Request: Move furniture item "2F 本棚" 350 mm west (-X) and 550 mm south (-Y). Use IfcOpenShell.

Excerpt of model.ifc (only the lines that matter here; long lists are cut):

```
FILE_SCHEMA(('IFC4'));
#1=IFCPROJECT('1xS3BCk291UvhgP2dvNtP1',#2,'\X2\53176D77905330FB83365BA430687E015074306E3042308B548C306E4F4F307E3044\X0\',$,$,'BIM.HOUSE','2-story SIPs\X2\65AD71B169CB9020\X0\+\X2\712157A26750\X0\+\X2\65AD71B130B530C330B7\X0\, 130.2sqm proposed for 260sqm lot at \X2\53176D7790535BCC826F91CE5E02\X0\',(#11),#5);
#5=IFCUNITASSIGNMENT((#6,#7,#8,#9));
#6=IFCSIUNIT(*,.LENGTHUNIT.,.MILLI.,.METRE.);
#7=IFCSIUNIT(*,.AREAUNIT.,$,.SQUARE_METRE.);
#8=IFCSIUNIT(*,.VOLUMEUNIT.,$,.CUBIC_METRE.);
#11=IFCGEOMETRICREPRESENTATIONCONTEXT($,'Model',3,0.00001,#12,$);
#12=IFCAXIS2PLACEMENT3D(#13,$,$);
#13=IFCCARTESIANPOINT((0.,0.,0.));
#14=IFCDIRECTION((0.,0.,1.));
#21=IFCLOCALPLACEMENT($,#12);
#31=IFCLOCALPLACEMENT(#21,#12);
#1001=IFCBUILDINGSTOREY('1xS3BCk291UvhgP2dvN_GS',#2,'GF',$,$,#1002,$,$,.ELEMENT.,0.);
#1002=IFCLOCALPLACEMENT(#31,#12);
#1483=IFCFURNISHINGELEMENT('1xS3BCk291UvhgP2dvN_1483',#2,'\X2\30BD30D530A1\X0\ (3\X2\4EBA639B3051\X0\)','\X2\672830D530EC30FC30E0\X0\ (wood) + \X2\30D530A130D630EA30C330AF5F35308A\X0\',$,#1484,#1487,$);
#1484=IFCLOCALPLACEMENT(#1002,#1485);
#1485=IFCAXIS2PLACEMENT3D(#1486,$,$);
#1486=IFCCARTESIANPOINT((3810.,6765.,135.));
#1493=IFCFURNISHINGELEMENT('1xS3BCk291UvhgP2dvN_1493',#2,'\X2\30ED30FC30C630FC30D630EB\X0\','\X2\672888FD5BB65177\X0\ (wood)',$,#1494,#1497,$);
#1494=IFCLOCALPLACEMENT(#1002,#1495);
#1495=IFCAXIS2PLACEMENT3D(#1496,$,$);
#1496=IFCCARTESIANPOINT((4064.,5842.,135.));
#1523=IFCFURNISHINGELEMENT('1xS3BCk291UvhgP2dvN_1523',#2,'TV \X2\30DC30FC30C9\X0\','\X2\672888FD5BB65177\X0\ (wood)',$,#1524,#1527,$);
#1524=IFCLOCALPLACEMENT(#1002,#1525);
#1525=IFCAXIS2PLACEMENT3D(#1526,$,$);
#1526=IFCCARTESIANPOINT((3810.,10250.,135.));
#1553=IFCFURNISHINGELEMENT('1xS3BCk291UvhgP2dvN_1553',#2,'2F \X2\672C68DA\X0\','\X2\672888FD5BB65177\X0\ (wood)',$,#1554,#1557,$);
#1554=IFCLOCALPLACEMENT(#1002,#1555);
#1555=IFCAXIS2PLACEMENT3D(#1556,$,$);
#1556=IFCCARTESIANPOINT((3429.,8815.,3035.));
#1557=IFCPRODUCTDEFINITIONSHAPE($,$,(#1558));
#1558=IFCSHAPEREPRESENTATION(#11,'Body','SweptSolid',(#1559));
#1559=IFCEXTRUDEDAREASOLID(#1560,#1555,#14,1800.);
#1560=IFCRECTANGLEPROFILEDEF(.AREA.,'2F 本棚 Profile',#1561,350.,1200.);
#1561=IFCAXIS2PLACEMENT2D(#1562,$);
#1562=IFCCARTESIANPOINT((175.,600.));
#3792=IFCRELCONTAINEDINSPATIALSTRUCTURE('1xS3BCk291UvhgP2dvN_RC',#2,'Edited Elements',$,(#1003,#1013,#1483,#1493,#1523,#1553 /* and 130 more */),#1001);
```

```python
import ifcopenshell
import ifcopenshell.api.geometry
import ifcopenshell.util.placement
import ifcopenshell.util.unit

model = ifcopenshell.open("model.ifc")
unit_scale = ifcopenshell.util.unit.calculate_unit_scale(model)

item = model.by_guid("1xS3BCk291UvhgP2dvN_1553")
matrix = ifcopenshell.util.placement.get_local_placement(item.ObjectPlacement)
matrix[0, 3] -= 0.35 / unit_scale
matrix[1, 3] -= 0.55 / unit_scale
ifcopenshell.api.geometry.edit_object_placement(model, product=item, matrix=matrix, is_si=False)

print(ifcopenshell.util.placement.get_local_placement(item.ObjectPlacement).round(3) + 0.0)

model.write("model-out.ifc")
```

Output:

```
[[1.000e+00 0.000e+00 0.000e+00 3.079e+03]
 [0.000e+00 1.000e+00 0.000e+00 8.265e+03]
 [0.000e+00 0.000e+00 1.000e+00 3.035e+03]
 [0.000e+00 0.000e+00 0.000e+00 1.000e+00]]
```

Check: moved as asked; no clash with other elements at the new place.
